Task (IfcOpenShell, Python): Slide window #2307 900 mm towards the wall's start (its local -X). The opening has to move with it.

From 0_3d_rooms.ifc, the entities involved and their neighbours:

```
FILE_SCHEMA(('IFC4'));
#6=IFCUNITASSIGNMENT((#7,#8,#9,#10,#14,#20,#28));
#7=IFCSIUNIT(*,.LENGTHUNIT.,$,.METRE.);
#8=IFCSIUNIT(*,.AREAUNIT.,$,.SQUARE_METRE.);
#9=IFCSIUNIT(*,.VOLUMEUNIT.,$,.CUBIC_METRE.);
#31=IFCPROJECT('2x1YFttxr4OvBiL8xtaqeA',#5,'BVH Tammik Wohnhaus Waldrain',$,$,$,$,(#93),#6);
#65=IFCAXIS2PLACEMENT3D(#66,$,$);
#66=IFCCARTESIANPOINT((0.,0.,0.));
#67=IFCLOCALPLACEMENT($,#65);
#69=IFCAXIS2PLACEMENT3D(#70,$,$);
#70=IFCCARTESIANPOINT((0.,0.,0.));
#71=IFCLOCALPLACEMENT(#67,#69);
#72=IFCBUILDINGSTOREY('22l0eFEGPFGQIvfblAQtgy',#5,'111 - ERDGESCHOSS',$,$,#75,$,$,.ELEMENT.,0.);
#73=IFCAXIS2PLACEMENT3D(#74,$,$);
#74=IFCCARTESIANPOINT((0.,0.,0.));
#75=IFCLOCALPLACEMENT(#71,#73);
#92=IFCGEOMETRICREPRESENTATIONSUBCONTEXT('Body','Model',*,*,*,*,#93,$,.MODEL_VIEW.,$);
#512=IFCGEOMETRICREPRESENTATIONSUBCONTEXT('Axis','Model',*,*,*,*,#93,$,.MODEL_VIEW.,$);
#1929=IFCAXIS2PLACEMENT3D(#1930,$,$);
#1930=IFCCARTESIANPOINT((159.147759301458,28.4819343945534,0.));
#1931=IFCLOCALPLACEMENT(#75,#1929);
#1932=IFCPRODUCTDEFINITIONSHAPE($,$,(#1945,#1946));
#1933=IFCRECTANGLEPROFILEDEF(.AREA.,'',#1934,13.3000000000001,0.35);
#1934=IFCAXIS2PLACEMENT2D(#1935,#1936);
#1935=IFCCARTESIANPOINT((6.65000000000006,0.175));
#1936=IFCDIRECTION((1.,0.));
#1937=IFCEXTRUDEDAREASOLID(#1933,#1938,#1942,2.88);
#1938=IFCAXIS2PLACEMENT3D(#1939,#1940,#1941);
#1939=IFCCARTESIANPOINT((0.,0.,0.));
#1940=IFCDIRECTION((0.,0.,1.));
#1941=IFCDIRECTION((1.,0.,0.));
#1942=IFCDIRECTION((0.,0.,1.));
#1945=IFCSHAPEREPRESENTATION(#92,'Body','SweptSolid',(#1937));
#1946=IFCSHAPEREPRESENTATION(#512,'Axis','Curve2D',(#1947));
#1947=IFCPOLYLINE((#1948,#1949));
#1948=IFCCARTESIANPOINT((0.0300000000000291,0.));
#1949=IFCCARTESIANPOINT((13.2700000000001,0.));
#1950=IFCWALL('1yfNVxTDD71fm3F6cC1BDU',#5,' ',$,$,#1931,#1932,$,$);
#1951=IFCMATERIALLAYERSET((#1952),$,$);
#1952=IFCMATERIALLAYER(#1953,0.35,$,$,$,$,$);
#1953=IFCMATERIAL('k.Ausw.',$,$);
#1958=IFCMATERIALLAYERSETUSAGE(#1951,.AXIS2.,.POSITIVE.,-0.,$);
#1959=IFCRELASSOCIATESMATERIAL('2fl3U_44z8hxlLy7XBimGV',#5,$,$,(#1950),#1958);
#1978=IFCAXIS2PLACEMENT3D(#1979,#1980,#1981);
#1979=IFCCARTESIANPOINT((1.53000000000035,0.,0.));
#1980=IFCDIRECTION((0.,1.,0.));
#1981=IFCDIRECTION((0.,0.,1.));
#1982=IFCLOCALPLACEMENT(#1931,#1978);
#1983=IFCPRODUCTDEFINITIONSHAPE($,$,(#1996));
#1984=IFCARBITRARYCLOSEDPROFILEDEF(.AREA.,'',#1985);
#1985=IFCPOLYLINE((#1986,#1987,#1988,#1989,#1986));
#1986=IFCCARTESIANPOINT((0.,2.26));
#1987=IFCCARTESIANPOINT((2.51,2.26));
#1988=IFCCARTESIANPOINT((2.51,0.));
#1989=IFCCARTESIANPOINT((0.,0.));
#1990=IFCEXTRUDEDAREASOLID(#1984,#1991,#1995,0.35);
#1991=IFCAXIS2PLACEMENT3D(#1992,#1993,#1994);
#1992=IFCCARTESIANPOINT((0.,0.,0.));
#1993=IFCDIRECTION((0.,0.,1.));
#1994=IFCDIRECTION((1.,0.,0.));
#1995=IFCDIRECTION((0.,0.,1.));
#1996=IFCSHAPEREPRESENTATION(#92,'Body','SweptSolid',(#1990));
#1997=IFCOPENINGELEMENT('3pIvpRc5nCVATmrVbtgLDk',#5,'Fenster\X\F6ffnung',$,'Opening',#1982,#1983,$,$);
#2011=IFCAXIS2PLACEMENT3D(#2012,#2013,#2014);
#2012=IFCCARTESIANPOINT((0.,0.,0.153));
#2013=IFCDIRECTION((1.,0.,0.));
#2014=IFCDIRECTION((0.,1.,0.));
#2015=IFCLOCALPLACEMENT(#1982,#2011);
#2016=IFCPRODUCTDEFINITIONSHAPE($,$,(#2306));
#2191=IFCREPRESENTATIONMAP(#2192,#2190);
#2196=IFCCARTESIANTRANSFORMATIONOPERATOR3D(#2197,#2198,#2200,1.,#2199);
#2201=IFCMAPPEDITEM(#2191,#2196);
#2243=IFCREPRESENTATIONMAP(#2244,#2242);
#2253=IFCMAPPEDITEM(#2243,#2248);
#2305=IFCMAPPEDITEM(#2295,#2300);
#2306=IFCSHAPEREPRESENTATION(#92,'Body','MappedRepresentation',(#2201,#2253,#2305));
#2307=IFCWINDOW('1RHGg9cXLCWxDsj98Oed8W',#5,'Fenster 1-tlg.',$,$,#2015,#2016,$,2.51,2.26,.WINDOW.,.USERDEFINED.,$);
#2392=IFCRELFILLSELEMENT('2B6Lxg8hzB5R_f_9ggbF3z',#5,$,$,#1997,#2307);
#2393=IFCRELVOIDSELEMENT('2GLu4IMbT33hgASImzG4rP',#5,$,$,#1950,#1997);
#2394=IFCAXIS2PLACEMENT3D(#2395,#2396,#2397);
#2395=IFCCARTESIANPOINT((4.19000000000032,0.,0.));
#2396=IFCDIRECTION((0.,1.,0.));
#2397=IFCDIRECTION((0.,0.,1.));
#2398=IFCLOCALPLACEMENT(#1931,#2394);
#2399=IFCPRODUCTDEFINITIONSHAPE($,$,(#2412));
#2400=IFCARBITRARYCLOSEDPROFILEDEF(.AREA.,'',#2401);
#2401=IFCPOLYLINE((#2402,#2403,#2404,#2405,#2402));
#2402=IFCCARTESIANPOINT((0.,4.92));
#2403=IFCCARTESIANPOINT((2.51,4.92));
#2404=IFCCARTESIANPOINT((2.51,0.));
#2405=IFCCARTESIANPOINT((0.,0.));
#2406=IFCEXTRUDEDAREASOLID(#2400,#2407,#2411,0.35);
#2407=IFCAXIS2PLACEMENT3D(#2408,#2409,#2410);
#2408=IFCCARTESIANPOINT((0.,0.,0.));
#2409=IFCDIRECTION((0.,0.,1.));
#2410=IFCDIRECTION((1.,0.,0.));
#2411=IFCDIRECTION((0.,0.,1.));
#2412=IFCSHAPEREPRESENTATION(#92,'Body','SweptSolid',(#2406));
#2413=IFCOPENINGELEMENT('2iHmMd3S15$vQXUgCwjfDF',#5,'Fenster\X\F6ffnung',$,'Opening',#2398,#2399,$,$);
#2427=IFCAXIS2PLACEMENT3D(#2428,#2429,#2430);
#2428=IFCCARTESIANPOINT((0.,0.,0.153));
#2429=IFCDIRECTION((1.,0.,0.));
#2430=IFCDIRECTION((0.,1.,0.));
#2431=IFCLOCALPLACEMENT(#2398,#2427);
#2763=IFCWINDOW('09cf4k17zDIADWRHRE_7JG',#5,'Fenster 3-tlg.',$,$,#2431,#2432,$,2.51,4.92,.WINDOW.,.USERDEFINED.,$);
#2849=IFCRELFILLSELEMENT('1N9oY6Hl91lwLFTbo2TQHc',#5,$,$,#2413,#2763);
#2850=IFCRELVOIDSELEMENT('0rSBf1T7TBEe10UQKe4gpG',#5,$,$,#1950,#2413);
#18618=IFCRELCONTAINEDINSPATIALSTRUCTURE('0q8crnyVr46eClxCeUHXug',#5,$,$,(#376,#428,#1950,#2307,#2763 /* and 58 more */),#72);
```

```python
import ifcopenshell
import ifcopenshell.api.geometry
import ifcopenshell.util.placement

model = ifcopenshell.open("0_3d_rooms.ifc")

window = model.by_id(2307)
opening = window.FillsVoids[0].RelatingOpeningElement
wall = opening.VoidsElements[0].RelatingBuildingElement

wall_matrix = ifcopenshell.util.placement.get_local_placement(wall.ObjectPlacement)
shift = wall_matrix[:3, 0] * -0.9
before = ifcopenshell.util.placement.get_local_placement(window.ObjectPlacement)[:3, 3].copy()

# The window is placed relative to its opening, so it follows when the opening moves.
matrix = ifcopenshell.util.placement.get_local_placement(opening.ObjectPlacement)
matrix[:3, 3] += shift
ifcopenshell.api.geometry.edit_object_placement(
    model, product=opening, matrix=matrix, is_si=False, should_transform_children=True
)

after = ifcopenshell.util.placement.get_local_placement(window.ObjectPlacement)[:3, 3]
print("window moved by", (after - before).round(3) + 0.0)

model.write("0_3d_rooms_rev.ifc")
```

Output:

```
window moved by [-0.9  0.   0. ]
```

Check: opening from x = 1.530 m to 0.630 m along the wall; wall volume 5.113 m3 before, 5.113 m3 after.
